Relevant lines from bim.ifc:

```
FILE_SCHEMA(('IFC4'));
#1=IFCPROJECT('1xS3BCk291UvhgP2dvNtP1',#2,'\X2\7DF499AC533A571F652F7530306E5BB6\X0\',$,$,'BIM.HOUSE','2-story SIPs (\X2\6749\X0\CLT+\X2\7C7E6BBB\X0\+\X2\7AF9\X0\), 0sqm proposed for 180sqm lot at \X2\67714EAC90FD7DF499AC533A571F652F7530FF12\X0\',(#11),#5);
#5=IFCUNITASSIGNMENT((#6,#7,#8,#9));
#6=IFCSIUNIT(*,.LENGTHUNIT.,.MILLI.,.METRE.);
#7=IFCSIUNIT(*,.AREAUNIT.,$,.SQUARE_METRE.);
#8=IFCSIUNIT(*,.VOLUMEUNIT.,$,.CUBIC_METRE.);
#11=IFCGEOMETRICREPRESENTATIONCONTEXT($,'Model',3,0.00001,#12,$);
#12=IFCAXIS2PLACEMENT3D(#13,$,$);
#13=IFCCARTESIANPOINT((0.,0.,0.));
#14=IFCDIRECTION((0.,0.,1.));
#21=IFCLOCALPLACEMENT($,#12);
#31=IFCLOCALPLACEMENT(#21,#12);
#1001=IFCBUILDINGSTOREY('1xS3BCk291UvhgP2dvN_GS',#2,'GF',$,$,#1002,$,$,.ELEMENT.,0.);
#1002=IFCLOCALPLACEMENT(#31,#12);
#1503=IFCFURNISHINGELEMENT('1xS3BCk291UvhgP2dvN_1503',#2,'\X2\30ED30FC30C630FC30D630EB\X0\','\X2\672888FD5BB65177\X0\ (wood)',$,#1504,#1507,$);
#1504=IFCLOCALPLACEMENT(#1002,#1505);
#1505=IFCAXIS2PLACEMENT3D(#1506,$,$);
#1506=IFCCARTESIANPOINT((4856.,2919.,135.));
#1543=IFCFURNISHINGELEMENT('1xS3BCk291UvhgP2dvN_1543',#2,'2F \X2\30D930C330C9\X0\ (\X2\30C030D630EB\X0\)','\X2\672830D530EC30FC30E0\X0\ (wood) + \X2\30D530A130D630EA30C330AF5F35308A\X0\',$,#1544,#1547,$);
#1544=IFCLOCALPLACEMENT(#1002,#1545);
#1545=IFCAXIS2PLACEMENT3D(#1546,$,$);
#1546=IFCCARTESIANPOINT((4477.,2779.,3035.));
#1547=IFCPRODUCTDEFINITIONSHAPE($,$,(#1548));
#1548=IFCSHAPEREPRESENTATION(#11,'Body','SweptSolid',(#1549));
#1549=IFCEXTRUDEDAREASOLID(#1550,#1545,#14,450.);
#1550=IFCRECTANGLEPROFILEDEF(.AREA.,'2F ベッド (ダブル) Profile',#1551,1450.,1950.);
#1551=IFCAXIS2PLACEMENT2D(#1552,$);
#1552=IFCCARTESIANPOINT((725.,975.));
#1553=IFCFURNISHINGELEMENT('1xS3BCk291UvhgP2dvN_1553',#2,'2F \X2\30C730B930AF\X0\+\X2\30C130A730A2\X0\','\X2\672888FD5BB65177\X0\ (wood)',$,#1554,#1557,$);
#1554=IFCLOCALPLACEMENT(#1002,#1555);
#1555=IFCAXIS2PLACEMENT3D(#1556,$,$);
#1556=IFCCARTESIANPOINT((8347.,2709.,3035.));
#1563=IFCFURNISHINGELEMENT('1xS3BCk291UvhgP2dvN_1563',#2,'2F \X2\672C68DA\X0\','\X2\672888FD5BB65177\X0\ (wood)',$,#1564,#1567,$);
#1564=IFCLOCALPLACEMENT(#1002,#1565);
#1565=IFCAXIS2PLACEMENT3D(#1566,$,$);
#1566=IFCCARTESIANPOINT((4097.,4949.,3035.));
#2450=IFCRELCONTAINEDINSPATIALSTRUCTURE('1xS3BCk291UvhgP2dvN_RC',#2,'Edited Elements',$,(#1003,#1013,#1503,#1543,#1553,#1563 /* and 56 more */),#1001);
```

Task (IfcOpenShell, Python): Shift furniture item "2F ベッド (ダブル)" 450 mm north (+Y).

```python
import ifcopenshell
import ifcopenshell.api.geometry
import ifcopenshell.util.placement
import ifcopenshell.util.unit

model = ifcopenshell.open("bim.ifc")
unit_scale = ifcopenshell.util.unit.calculate_unit_scale(model)

item = model.by_guid("1xS3BCk291UvhgP2dvN_1543")
matrix = ifcopenshell.util.placement.get_local_placement(item.ObjectPlacement)
matrix[1, 3] += 0.45 / unit_scale
ifcopenshell.api.geometry.edit_object_placement(model, product=item, matrix=matrix, is_si=False)

print(ifcopenshell.util.placement.get_local_placement(item.ObjectPlacement).round(3) + 0.0)

model.write("bim_updated.ifc")
```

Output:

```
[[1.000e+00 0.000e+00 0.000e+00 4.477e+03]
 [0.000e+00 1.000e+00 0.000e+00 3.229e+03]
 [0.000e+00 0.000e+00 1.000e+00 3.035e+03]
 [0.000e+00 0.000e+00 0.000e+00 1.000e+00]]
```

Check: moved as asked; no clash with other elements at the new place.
